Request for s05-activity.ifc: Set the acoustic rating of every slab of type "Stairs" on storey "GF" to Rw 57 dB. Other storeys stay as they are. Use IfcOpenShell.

First a look at what the model holds.

```python
import ifcopenshell
import ifcopenshell.util.element

model = ifcopenshell.open("s05-activity.ifc")
print(model.schema)
storey = next(s for s in model.by_type("IfcBuildingStorey") if s.Name == "GF")
slabs = [e for e in ifcopenshell.util.element.get_decomposition(storey) if e.is_a("IfcSlab")]
seen = {}
for e in slabs:
    element_type = ifcopenshell.util.element.get_type(e)
    key = (element_type.Name if element_type != e and element_type else None, ifcopenshell.util.element.get_pset(e, "Pset_SlabCommon", "AcousticRating"))
    seen[key] = seen.get(key, 0) + 1
for (name, value), count in sorted(seen.items(), key=str):
    print(count, "x", name, "|", value)
```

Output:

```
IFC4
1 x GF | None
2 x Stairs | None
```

```python
import ifcopenshell
import ifcopenshell.api.pset
import ifcopenshell.util.element

model = ifcopenshell.open("s05-activity.ifc")

storey = next(s for s in model.by_type("IfcBuildingStorey") if s.Name == "GF")
slabs = [e for e in ifcopenshell.util.element.get_decomposition(storey) if e.is_a("IfcSlab")]

count = 0
for e in slabs:
    element_type = ifcopenshell.util.element.get_type(e)
    if element_type in (None, e) or element_type.Name != "Stairs":
        continue
    # add_pset returns the element's existing set when there is one.
    pset = ifcopenshell.api.pset.add_pset(model, product=e, name="Pset_SlabCommon")
    ifcopenshell.api.pset.edit_pset(model, pset=pset, properties={"AcousticRating": "Rw 57 dB"})
    count += 1

print(count, "slabs updated")

model.write("s05-activity-out.ifc")
```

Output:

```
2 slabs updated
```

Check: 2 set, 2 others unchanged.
